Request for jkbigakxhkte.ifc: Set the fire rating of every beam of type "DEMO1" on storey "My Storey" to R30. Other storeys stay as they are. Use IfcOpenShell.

First a look at what the model holds.

```python
import ifcopenshell
import ifcopenshell.util.element

model = ifcopenshell.open("jkbigakxhkte.ifc")
print(model.schema)
storey = next(s for s in model.by_type("IfcBuildingStorey") if s.Name == "My Storey")
beams = [e for e in ifcopenshell.util.element.get_decomposition(storey) if e.is_a("IfcBeam")]
seen = {}
for e in beams:
    element_type = ifcopenshell.util.element.get_type(e)
    key = (element_type.Name if element_type != e and element_type else None, ifcopenshell.util.element.get_pset(e, "Pset_BeamCommon", "FireRating"))
    seen[key] = seen.get(key, 0) + 1
for (name, value), count in sorted(seen.items(), key=str):
    print(count, "x", name, "|", value)
```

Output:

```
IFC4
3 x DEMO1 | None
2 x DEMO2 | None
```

```python
import ifcopenshell
import ifcopenshell.api.pset
import ifcopenshell.util.element

model = ifcopenshell.open("jkbigakxhkte.ifc")

storey = next(s for s in model.by_type("IfcBuildingStorey") if s.Name == "My Storey")
beams = [e for e in ifcopenshell.util.element.get_decomposition(storey) if e.is_a("IfcBeam")]

count = 0
for e in beams:
    element_type = ifcopenshell.util.element.get_type(e)
    if element_type in (None, e) or element_type.Name != "DEMO1":
        continue
    # add_pset returns the element's existing set when there is one.
    pset = ifcopenshell.api.pset.add_pset(model, product=e, name="Pset_BeamCommon")
    ifcopenshell.api.pset.edit_pset(model, pset=pset, properties={"FireRating": "R30"})
    count += 1

print(count, "beams updated")

model.write("jkbigakxhkte_edited.ifc")
```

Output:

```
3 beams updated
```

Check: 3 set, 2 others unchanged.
